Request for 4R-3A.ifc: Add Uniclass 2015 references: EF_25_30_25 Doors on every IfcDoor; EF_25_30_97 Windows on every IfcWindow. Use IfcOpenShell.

First a look at what the model holds.

```python
import ifcopenshell

model = ifcopenshell.open("4R-3A.ifc")
print(model.schema)
print("classifications:", [c.Name for c in model.by_type("IfcClassification")])
for ifc_class in ("IfcDoor", "IfcRoof", "IfcStair", "IfcWall", "IfcWindow"):
    print(ifc_class, len(model.by_type(ifc_class)))
```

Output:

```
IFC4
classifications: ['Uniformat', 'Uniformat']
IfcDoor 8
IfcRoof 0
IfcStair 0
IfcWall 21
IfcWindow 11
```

```python
import ifcopenshell
import ifcopenshell.api.classification

model = ifcopenshell.open("4R-3A.ifc")

system = ifcopenshell.api.classification.add_classification(model, classification="Uniclass 2015")

codes = {
    "IfcDoor": ("EF_25_30_25", "Doors"),
    "IfcWindow": ("EF_25_30_97", "Windows"),
}
for ifc_class, (code, name) in codes.items():
    products = model.by_type(ifc_class)
    ifcopenshell.api.classification.add_reference(
        model, products=products, classification=system, identification=code, name=name
    )
    print(code, len(products))

model.write("4R-3A-out.ifc")
```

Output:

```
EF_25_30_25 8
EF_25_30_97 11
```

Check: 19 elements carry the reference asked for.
